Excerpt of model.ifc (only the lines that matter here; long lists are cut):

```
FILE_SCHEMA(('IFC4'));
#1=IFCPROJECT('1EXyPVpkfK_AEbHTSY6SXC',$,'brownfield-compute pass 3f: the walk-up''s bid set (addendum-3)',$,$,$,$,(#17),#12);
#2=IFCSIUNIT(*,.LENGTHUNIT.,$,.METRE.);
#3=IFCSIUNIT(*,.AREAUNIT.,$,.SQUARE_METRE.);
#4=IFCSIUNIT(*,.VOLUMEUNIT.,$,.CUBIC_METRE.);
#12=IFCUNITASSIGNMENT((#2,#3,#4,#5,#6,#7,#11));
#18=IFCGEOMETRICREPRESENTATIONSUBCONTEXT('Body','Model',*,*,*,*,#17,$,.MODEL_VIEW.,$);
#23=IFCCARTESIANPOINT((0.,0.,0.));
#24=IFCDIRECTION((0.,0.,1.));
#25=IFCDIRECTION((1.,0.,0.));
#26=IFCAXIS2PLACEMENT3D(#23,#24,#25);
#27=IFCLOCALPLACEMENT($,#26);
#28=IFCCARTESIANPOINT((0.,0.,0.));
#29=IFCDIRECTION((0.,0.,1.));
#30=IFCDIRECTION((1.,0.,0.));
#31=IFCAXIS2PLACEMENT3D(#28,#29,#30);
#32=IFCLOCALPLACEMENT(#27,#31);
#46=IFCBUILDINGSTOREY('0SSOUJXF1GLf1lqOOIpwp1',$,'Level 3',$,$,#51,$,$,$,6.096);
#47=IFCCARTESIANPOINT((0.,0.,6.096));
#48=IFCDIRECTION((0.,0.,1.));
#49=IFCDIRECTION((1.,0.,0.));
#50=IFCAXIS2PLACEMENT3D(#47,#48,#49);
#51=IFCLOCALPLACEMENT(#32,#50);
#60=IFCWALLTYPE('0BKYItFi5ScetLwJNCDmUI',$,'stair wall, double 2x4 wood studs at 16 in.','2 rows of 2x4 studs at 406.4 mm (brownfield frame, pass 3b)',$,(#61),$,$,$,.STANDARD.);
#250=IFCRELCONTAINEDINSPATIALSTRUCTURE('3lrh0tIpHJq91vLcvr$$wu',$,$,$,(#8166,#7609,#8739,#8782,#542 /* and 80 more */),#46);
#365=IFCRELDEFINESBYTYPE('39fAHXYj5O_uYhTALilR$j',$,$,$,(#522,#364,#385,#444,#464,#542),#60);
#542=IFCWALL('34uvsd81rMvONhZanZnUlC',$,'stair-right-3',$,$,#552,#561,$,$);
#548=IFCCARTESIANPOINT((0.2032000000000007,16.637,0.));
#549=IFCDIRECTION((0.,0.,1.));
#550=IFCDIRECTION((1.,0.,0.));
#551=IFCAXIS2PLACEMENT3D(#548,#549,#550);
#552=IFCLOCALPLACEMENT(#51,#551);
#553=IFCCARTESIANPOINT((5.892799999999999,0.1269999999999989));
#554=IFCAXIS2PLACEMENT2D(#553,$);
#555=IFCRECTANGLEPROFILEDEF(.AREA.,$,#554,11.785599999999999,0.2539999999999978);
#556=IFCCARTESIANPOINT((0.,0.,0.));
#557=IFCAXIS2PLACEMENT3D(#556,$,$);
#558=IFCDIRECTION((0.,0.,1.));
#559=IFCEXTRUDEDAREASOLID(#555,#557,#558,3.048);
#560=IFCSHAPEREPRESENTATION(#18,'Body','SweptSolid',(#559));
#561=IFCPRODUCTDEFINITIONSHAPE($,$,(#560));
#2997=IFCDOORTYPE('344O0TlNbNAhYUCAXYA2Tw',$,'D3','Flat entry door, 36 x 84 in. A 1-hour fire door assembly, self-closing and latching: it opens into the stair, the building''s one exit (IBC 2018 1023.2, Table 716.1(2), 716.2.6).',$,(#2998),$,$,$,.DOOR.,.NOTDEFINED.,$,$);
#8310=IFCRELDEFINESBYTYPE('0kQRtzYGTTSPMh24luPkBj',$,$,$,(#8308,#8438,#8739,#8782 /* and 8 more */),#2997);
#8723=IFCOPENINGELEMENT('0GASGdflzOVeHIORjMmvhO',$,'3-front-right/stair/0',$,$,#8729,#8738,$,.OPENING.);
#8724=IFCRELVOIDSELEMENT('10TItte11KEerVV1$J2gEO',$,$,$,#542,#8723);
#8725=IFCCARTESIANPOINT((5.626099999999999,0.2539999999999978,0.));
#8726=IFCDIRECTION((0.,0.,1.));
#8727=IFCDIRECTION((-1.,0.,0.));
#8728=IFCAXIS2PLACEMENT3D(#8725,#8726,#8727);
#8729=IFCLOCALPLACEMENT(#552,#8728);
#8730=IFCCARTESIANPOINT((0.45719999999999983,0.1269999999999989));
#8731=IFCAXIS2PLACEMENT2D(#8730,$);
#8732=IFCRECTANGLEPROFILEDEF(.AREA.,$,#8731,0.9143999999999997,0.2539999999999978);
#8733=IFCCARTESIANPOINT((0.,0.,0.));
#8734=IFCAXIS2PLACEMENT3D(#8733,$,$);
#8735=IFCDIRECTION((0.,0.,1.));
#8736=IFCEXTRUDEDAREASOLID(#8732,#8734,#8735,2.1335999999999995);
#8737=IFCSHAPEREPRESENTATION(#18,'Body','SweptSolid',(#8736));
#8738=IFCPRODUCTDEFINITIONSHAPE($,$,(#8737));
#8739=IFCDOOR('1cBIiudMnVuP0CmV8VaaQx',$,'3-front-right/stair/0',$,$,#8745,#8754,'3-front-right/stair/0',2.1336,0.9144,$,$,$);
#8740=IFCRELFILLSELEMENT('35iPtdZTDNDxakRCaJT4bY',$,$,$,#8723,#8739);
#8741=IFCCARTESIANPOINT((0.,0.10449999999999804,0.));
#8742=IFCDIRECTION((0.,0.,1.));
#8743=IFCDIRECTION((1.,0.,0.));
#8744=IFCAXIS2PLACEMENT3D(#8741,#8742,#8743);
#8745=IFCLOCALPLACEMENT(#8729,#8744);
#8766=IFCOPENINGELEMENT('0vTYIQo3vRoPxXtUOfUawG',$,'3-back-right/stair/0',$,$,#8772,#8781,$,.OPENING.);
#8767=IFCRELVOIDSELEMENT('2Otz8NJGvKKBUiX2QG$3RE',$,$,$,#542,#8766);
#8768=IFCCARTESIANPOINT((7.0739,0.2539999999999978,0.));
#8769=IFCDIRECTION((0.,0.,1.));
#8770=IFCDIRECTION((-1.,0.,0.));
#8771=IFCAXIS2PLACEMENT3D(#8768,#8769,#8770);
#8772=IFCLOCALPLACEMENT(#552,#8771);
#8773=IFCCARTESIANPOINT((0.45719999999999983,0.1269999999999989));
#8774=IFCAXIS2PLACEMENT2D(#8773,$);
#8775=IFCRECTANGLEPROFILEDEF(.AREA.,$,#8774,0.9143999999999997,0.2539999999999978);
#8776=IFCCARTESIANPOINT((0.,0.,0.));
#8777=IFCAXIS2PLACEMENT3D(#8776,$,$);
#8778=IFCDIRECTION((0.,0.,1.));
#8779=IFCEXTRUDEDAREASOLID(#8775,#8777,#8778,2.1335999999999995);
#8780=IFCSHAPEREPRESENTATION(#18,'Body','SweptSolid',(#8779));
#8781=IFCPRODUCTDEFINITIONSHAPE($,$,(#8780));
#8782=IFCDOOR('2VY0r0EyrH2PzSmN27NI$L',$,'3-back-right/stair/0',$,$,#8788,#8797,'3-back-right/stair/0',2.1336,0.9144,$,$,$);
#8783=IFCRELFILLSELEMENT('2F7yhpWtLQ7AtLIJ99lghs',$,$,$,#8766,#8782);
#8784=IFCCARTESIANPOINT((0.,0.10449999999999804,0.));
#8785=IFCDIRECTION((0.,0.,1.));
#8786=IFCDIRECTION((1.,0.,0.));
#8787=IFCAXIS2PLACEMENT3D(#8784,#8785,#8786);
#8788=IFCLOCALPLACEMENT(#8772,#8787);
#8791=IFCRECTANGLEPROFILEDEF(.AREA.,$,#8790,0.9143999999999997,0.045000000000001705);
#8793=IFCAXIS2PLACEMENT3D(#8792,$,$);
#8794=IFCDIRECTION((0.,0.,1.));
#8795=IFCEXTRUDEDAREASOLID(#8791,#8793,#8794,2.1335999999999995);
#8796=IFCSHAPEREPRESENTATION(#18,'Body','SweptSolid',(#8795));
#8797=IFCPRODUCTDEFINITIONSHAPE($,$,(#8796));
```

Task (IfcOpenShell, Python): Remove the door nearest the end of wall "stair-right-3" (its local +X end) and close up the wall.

```python
import ifcopenshell
import ifcopenshell.api.feature
import ifcopenshell.api.root
import ifcopenshell.geom
import ifcopenshell.util.shape

model = ifcopenshell.open("model.ifc")
settings = ifcopenshell.geom.settings()


def volume(element):
    """Net volume in cubic metres, openings subtracted."""
    shape = ifcopenshell.geom.create_shape(settings, element)
    return ifcopenshell.util.shape.get_volume(shape.geometry)


door = model.by_id(8782)
opening = door.FillsVoids[0].RelatingOpeningElement
wall = opening.VoidsElements[0].RelatingBuildingElement
before = volume(wall)

ifcopenshell.api.root.remove_product(model, product=door)
ifcopenshell.api.feature.remove_feature(model, feature=opening)

after = volume(wall)

print(f"wall volume {before:.3f} -> {after:.3f} m3")

model.write("model_rev.ifc")
```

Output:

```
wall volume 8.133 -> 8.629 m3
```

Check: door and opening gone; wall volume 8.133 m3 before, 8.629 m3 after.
